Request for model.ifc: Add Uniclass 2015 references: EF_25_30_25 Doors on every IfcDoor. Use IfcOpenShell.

First a look at what the model holds.

```python
import ifcopenshell

model = ifcopenshell.open("model.ifc")
print(model.schema)
print("classifications:", [c.Name for c in model.by_type("IfcClassification")])
for ifc_class in ("IfcDoor", "IfcRoof", "IfcStair", "IfcWall", "IfcWindow"):
    print(ifc_class, len(model.by_type(ifc_class)))
```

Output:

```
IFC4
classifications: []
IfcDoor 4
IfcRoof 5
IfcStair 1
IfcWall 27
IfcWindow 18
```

```python
import ifcopenshell
import ifcopenshell.api.classification

model = ifcopenshell.open("model.ifc")

system = ifcopenshell.api.classification.add_classification(model, classification="Uniclass 2015")

codes = {
    "IfcDoor": ("EF_25_30_25", "Doors"),
}
for ifc_class, (code, name) in codes.items():
    products = model.by_type(ifc_class)
    ifcopenshell.api.classification.add_reference(
        model, products=products, classification=system, identification=code, name=name
    )
    print(code, len(products))

model.write("model_updated.ifc")
```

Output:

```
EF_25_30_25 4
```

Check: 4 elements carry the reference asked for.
